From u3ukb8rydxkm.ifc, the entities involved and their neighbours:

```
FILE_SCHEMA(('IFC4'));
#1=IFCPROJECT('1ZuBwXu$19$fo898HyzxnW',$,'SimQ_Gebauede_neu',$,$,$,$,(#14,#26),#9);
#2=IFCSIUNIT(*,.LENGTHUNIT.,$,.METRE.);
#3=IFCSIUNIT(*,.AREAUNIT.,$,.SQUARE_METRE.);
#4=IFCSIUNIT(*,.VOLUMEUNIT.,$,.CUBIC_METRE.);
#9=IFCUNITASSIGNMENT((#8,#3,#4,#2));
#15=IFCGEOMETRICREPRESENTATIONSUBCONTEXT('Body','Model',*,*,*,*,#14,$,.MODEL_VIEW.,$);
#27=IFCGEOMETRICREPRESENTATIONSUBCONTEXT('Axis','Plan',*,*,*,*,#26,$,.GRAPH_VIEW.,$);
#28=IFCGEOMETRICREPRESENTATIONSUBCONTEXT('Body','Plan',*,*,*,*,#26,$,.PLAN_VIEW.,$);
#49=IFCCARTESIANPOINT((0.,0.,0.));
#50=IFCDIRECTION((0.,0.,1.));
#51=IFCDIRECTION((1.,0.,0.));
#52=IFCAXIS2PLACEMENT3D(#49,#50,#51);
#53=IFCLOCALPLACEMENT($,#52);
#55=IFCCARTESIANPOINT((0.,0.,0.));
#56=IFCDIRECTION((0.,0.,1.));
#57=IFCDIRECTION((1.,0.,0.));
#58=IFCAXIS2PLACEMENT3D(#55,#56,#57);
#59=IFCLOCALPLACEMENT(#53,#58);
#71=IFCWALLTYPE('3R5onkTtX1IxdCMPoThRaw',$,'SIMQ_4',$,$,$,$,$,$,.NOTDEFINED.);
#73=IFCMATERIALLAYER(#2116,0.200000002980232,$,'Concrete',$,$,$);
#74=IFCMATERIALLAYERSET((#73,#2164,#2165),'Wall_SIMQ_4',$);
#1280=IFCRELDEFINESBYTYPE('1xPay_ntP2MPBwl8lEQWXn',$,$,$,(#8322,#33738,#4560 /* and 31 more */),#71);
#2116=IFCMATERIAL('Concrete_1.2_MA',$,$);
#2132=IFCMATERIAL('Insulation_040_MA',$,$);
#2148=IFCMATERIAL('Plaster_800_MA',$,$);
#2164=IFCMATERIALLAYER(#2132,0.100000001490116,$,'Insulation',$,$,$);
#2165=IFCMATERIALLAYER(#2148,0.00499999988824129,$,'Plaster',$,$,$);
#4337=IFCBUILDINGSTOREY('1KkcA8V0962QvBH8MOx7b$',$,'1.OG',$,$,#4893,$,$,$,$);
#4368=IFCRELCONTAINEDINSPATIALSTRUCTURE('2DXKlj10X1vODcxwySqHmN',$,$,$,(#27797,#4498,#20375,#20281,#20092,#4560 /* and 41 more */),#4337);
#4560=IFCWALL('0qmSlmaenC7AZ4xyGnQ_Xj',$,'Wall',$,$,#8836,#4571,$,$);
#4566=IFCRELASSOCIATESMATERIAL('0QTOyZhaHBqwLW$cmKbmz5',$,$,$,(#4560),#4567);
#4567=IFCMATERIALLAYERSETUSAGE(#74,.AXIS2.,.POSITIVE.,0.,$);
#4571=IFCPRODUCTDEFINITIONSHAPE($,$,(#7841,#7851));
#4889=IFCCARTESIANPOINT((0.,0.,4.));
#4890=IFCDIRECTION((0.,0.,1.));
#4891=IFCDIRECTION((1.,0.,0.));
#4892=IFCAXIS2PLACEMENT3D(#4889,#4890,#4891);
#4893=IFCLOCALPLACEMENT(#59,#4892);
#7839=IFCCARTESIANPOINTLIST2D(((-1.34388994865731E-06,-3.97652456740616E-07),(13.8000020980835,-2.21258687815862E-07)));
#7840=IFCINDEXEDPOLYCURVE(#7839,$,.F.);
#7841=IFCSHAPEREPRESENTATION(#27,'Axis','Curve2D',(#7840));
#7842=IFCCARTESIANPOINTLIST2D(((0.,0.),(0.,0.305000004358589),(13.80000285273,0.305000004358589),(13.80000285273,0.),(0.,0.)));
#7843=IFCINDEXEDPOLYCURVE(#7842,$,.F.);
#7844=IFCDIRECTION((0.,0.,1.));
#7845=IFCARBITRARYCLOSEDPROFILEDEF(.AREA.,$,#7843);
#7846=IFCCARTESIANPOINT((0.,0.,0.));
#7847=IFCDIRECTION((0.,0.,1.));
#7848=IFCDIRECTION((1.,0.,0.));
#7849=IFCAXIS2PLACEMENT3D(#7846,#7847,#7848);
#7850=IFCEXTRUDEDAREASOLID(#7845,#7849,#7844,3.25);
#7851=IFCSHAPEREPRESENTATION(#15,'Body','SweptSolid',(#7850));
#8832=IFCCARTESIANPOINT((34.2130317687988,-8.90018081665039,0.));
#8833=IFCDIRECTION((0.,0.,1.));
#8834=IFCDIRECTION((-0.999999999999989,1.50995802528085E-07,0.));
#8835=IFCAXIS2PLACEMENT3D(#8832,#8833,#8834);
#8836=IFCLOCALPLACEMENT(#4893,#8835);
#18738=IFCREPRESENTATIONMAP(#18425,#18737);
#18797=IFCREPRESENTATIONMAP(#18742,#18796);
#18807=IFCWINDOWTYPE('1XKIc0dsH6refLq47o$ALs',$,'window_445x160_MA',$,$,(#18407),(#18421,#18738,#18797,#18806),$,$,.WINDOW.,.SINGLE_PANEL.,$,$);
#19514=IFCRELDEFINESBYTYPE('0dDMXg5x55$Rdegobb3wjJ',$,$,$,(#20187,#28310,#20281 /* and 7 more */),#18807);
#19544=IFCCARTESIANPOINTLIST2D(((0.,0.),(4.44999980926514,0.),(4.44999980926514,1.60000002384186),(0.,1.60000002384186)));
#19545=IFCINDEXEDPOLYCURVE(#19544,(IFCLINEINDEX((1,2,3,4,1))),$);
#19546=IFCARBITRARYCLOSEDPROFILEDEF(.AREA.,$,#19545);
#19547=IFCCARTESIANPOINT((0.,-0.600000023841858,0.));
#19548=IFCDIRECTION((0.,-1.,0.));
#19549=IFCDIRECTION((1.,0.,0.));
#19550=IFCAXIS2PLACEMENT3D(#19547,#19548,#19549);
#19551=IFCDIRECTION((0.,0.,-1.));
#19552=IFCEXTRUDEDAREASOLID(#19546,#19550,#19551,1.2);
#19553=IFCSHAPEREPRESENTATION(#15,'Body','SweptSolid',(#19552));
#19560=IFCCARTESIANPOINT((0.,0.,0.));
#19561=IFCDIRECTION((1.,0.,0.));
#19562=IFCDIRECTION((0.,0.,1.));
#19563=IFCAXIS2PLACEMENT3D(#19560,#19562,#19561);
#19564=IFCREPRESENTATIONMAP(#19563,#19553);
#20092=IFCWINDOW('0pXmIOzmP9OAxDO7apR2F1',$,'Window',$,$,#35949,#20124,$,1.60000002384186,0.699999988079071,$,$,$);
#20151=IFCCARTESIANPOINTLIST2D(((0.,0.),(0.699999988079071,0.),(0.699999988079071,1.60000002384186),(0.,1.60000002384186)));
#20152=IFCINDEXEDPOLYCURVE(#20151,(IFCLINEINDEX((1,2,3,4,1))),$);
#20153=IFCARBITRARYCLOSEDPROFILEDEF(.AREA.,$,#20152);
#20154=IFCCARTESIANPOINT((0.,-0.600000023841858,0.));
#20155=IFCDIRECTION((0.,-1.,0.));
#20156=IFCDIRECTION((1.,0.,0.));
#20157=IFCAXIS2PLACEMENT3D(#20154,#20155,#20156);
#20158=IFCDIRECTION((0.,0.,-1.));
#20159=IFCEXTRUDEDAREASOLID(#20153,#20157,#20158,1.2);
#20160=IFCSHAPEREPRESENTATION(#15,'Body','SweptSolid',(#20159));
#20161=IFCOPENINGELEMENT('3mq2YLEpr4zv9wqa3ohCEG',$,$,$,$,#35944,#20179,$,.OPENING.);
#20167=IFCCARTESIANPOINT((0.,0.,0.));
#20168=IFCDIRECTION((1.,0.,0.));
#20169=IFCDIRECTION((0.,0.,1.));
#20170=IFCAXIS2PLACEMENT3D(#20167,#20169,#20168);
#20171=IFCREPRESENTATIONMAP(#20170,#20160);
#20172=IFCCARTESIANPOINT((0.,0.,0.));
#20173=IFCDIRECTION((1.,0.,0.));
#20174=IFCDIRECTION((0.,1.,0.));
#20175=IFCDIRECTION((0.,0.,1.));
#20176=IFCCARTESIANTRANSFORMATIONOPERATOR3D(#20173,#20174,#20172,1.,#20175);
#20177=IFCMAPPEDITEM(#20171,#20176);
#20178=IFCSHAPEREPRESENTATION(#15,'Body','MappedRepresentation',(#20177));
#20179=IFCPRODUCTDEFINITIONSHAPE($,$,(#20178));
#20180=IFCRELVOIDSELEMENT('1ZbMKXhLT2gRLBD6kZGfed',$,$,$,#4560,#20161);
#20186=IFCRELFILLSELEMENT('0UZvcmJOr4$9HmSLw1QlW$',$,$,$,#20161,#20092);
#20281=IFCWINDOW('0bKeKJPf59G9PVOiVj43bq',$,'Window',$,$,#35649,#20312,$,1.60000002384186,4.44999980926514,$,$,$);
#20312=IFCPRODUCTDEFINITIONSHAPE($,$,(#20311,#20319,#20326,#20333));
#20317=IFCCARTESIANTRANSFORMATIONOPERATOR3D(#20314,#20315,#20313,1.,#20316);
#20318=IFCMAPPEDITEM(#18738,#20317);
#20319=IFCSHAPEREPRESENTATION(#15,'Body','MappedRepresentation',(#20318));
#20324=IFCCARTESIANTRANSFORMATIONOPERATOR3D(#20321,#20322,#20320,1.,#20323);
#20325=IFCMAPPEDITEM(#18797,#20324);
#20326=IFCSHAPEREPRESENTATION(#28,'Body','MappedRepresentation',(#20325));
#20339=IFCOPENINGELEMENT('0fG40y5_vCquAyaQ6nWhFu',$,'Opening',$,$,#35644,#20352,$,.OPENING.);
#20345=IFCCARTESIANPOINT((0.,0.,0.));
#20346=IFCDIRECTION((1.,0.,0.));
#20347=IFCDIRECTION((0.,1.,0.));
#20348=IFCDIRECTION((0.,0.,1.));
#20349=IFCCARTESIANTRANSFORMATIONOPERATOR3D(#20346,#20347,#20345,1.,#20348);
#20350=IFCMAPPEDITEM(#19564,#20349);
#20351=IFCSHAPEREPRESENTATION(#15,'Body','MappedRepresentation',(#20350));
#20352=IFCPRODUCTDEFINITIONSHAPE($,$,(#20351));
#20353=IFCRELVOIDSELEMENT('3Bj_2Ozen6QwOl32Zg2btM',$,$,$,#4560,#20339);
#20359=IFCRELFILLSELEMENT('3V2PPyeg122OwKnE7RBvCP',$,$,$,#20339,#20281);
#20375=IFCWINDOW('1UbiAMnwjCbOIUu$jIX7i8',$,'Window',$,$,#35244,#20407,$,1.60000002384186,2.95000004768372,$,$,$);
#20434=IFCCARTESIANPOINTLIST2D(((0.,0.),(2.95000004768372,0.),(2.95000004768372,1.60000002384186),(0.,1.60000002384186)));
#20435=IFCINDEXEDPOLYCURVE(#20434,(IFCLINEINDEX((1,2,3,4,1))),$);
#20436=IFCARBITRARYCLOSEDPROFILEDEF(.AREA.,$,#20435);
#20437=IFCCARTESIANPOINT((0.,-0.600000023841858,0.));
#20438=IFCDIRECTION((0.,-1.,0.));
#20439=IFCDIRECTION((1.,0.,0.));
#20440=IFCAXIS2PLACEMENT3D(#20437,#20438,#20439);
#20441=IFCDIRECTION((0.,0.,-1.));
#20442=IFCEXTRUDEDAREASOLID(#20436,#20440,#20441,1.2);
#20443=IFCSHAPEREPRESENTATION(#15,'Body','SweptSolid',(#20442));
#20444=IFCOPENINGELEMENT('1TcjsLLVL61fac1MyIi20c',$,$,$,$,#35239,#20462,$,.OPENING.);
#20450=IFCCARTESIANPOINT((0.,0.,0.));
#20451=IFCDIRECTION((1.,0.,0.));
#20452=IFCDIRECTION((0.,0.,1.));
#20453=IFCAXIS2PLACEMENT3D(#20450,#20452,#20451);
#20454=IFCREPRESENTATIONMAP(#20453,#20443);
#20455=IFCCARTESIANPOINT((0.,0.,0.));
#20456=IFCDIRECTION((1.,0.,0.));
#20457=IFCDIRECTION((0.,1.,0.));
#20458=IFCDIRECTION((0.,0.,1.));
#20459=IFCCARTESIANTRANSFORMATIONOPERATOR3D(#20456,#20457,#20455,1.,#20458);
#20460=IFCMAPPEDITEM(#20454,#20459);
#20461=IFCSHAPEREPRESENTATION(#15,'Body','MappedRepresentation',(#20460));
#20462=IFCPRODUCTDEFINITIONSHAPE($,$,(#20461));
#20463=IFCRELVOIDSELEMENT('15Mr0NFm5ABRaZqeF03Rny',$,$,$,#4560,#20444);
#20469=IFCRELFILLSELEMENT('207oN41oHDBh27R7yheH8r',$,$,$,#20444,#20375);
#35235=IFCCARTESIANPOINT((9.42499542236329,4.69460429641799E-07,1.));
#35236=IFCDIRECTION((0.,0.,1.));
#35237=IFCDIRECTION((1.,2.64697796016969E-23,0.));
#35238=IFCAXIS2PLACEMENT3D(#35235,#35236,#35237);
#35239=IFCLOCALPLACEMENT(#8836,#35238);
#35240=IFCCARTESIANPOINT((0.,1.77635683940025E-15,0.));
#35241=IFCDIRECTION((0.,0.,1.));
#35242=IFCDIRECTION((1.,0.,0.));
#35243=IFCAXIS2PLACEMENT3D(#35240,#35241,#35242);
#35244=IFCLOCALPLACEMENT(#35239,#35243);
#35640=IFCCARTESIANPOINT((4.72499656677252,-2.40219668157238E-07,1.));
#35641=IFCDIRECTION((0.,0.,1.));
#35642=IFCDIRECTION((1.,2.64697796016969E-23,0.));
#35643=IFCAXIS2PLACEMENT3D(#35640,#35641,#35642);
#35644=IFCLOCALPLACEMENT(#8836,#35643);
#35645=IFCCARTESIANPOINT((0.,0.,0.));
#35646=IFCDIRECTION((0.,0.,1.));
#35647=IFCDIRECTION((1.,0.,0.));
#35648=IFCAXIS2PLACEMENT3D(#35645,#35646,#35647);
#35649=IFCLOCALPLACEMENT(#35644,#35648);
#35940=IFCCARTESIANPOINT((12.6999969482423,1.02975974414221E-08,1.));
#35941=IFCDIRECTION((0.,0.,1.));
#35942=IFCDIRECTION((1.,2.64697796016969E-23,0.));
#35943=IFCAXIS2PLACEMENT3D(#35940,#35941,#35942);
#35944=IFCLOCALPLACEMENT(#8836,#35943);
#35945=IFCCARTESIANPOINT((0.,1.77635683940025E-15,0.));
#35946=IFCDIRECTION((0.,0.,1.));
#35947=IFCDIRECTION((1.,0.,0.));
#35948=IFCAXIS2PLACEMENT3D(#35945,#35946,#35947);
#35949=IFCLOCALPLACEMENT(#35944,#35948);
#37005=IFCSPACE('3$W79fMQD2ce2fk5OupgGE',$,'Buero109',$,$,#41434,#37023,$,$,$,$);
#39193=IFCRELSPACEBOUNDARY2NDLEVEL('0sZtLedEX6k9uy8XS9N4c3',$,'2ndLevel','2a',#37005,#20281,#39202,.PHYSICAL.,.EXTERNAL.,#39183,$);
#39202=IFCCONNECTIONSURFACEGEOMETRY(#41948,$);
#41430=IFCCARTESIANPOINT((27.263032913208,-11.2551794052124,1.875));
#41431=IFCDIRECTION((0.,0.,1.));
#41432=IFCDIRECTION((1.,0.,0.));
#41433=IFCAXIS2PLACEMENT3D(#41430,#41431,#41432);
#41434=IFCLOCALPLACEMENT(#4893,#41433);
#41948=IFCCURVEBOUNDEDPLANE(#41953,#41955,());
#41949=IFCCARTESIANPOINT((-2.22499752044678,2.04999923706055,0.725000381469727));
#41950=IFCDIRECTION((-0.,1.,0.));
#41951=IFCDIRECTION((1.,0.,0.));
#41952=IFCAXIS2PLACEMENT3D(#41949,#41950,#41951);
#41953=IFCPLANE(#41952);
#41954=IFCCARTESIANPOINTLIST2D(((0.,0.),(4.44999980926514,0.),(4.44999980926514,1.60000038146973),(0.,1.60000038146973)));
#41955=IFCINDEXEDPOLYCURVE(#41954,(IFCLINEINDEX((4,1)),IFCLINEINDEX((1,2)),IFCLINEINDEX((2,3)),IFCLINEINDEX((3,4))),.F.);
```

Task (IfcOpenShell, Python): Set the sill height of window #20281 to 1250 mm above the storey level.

```python
import numpy as np
import ifcopenshell
import ifcopenshell.api.geometry
import ifcopenshell.geom
import ifcopenshell.util.element
import ifcopenshell.util.placement
import ifcopenshell.util.shape
import ifcopenshell.util.unit

model = ifcopenshell.open("u3ukb8rydxkm.ifc")
unit_scale = ifcopenshell.util.unit.calculate_unit_scale(model)

window = model.by_guid("0bKeKJPf59G9PVOiVj43bq")
opening = window.FillsVoids[0].RelatingOpeningElement
storey = ifcopenshell.util.element.get_container(window, ifc_class="IfcBuildingStorey")
level = ifcopenshell.util.placement.get_local_placement(storey.ObjectPlacement)[2, 3]

# The opening's origin need not be at the sill, so measure its lowest point.
shape = ifcopenshell.geom.create_shape(ifcopenshell.geom.settings(), opening)
bottom = ifcopenshell.util.shape.get_shape_bottom_elevation(shape, shape.geometry) / unit_scale
dz = level + 1.25 / unit_scale - bottom

shift = np.array([0.0, 0.0, dz])
# The window is placed relative to its opening, so it follows when the opening moves.
matrix = ifcopenshell.util.placement.get_local_placement(opening.ObjectPlacement)
matrix[:3, 3] += shift
ifcopenshell.api.geometry.edit_object_placement(
    model, product=opening, matrix=matrix, is_si=False, should_transform_children=True
)

# Space boundary surfaces are stored in each space's coordinates; move them too.
for rel in window.ProvidesBoundaries:
    if not rel.ConnectionGeometry:
        continue
    surface = rel.ConnectionGeometry.SurfaceOnRelatingElement.BasisSurface
    space_matrix = ifcopenshell.util.placement.get_local_placement(rel.RelatingSpace.ObjectPlacement)
    point = np.array(surface.Position.Location.Coordinates) + space_matrix[:3, :3].T @ shift
    surface.Position = model.createIfcAxis2Placement3D(
        model.createIfcCartesianPoint(point.tolist()), surface.Position.Axis, surface.Position.RefDirection
    )

print(f"moved by {dz * unit_scale:+.3f} m")

model.write("u3ukb8rydxkm_v2.ifc")
```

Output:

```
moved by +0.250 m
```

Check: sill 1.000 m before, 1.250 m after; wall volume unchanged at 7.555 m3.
